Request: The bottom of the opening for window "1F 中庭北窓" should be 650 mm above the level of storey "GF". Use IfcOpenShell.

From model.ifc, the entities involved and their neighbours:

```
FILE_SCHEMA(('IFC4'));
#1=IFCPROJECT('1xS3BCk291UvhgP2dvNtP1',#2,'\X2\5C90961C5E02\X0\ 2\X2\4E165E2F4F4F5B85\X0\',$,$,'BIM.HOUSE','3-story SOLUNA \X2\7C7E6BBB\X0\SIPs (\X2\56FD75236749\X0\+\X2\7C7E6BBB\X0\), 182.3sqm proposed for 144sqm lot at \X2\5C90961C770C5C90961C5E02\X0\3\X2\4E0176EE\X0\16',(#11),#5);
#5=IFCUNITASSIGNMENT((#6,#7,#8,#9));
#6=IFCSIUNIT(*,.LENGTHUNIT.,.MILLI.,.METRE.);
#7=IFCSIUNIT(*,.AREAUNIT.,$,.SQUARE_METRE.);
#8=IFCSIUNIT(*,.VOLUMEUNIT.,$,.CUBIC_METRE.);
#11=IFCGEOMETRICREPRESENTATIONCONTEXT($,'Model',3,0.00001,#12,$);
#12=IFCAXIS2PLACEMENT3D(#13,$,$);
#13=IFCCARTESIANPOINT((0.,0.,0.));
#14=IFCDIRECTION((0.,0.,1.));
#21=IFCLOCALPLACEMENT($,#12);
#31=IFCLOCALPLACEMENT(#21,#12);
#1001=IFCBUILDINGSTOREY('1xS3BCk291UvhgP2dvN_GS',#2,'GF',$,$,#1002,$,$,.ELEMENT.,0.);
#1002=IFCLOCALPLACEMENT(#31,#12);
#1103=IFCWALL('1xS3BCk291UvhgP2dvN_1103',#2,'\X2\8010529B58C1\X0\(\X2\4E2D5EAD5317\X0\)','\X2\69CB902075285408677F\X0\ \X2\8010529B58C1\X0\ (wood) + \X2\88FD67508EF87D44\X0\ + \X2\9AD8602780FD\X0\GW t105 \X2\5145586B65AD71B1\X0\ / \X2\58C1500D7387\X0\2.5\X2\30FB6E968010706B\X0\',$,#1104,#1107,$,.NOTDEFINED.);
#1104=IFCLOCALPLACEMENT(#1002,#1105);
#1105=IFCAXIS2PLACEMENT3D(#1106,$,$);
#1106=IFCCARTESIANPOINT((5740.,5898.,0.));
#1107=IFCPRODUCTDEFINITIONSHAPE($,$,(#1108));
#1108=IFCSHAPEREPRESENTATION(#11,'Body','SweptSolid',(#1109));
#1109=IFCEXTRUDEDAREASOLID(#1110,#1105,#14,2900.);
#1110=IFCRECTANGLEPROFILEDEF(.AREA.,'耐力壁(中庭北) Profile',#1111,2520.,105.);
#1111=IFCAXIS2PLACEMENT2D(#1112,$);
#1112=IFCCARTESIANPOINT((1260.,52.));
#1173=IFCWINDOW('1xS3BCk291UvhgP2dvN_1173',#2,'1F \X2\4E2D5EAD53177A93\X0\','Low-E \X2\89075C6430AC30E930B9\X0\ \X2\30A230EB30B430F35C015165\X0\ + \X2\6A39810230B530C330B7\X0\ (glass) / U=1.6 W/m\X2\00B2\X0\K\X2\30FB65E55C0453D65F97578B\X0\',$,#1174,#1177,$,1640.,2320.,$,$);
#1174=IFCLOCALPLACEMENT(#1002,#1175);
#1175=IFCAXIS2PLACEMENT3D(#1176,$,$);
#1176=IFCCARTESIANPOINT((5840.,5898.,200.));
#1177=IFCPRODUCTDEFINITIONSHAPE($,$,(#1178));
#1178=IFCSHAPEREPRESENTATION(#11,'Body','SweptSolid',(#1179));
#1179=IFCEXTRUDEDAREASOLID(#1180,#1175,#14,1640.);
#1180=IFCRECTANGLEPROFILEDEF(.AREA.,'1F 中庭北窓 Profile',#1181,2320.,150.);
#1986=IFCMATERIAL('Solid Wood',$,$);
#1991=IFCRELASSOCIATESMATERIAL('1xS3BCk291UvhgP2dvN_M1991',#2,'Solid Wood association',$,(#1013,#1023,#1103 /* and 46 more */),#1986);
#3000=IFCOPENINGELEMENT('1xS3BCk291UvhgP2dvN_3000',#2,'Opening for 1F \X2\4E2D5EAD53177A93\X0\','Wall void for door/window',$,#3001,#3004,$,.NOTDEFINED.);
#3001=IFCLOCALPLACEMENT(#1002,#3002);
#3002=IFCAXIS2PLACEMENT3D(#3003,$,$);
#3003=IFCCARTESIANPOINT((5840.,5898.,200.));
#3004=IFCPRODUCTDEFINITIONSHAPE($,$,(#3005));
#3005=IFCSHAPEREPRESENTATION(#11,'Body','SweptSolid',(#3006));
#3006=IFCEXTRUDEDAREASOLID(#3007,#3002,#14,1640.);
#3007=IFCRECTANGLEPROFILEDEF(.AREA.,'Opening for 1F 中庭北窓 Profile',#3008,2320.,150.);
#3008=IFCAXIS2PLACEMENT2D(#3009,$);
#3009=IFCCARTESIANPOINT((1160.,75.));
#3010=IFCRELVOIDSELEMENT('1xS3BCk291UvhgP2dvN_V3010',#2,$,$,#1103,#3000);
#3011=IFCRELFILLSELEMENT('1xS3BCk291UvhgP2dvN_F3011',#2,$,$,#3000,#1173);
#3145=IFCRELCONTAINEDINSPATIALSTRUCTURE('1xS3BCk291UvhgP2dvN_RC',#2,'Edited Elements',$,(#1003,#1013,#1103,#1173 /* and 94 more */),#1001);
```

```python
import numpy as np
import ifcopenshell
import ifcopenshell.api.geometry
import ifcopenshell.geom
import ifcopenshell.util.element
import ifcopenshell.util.placement
import ifcopenshell.util.shape
import ifcopenshell.util.unit

model = ifcopenshell.open("model.ifc")
unit_scale = ifcopenshell.util.unit.calculate_unit_scale(model)

window = model.by_guid("1xS3BCk291UvhgP2dvN_1173")
opening = window.FillsVoids[0].RelatingOpeningElement
storey = ifcopenshell.util.element.get_container(window, ifc_class="IfcBuildingStorey")
level = ifcopenshell.util.placement.get_local_placement(storey.ObjectPlacement)[2, 3]

# The opening's origin need not be at the sill, so measure its lowest point.
shape = ifcopenshell.geom.create_shape(ifcopenshell.geom.settings(), opening)
bottom = ifcopenshell.util.shape.get_shape_bottom_elevation(shape, shape.geometry) / unit_scale
dz = level + 650.0 - bottom

shift = np.array([0.0, 0.0, dz])
# The window is not placed relative to its opening, so move both.
for product in (opening, window):
    matrix = ifcopenshell.util.placement.get_local_placement(product.ObjectPlacement)
    matrix[:3, 3] += shift
    ifcopenshell.api.geometry.edit_object_placement(model, product=product, matrix=matrix, is_si=False)

print(f"moved by {dz * unit_scale:+.3f} m")

model.write("model-out.ifc")
```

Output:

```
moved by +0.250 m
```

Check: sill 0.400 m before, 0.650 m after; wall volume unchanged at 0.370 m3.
